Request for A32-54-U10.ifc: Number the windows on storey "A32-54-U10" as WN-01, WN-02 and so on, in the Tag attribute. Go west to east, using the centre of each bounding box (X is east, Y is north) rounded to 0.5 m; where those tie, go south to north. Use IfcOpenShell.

First a look at what the model holds.

```python
import ifcopenshell
import ifcopenshell.util.element
import ifcopenshell.util.placement

model = ifcopenshell.open("A32-54-U10.ifc")
print(model.schema)
storey = next(s for s in model.by_type("IfcBuildingStorey") if s.Name == "A32-54-U10")
windows = [e for e in ifcopenshell.util.element.get_decomposition(storey) if e.is_a("IfcWindow")]
for e in sorted(windows, key=lambda e: e.id()):
    origin = ifcopenshell.util.placement.get_local_placement(e.ObjectPlacement)[:3, 3]
    print(e.id(), e.Tag, e.Name, origin.round(2) + 0.0, sep=" | ")
```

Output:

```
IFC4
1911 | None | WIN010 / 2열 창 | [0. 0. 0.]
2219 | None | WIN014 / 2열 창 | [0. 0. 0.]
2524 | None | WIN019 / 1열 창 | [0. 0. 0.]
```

```python
import ifcopenshell
import ifcopenshell.geom
import ifcopenshell.util.element
import ifcopenshell.util.shape

model = ifcopenshell.open("A32-54-U10.ifc")
settings = ifcopenshell.geom.settings()
settings.set("use-world-coords", True)


def centre(element):
    shape = ifcopenshell.geom.create_shape(settings, element)
    return ifcopenshell.util.shape.get_bbox_centroid(shape.geometry)


storey = next(s for s in model.by_type("IfcBuildingStorey") if s.Name == "A32-54-U10")
windows = [e for e in ifcopenshell.util.element.get_decomposition(storey) if e.is_a("IfcWindow")]

# Insertion points can sit at a corner or the storey origin, so sort by the geometry (in metres).
centres = {e: centre(e) for e in windows}
windows.sort(key=lambda e: (round(centres[e][0] / 0.5), centres[e][1]))

for i, e in enumerate(windows, start=1):
    number = f"WN-{i:02d}"
    e.Tag = number
    print(e.id(), number)

model.write("A32-54-U10_updated.ifc")
```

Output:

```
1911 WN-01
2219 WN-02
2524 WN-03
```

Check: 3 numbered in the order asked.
